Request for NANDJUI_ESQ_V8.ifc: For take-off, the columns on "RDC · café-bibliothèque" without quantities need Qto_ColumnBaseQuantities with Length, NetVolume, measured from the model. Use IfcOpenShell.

First a look at what the model holds.

```python
import ifcopenshell
import ifcopenshell.util.element
import ifcopenshell.util.unit

model = ifcopenshell.open("NANDJUI_ESQ_V8.ifc")
print(model.schema)
for unit_type in ("LENGTHUNIT", "AREAUNIT", "VOLUMEUNIT"):
    print(unit_type, ifcopenshell.util.unit.calculate_unit_scale(model, unit_type))
storey = next(s for s in model.by_type("IfcBuildingStorey") if s.Name == "RDC · café-bibliothèque")
columns = [e for e in ifcopenshell.util.element.get_decomposition(storey) if e.is_a("IfcColumn")]
for e in sorted(columns, key=lambda e: e.id()):
    print(e.id(), e.is_a(), e.Name, list(ifcopenshell.util.element.get_psets(e, qtos_only=True)), sep=" | ")
```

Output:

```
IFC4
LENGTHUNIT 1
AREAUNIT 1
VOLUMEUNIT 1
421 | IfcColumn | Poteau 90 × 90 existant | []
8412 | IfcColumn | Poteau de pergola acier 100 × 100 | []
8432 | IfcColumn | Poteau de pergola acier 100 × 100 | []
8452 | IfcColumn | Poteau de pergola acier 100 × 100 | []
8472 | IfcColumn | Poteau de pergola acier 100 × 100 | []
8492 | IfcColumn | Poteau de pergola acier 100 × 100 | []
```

```python
import ifcopenshell
import ifcopenshell.api.pset
import ifcopenshell.geom
import ifcopenshell.util.element
import ifcopenshell.util.shape
import ifcopenshell.util.unit

model = ifcopenshell.open("NANDJUI_ESQ_V8.ifc")
unit_scale = ifcopenshell.util.unit.calculate_unit_scale(model)
volume_scale = ifcopenshell.util.unit.calculate_unit_scale(model, "VOLUMEUNIT")
settings = ifcopenshell.geom.settings()

storey = next(s for s in model.by_type("IfcBuildingStorey") if s.Name == "RDC · café-bibliothèque")
columns = [e for e in ifcopenshell.util.element.get_decomposition(storey) if e.is_a("IfcColumn")]

for e in sorted(columns, key=lambda e: e.id()):
    if ifcopenshell.util.element.get_psets(e, qtos_only=True, should_inherit=False):
        continue
    # Geometry comes back in metres, in the element's own axes.
    shape = ifcopenshell.geom.create_shape(settings, e)
    values = {
        "Length": ifcopenshell.util.shape.get_z(shape.geometry) / unit_scale,
        "NetVolume": ifcopenshell.util.shape.get_volume(shape.geometry) / volume_scale,
    }
    qto = ifcopenshell.api.pset.add_qto(model, product=e, name="Qto_ColumnBaseQuantities")
    ifcopenshell.api.pset.edit_qto(model, qto=qto, properties=values)
    print(e.id(), {k: round(v, 3) for k, v in values.items()})

model.write("NANDJUI_ESQ_V8_edited.ifc")
```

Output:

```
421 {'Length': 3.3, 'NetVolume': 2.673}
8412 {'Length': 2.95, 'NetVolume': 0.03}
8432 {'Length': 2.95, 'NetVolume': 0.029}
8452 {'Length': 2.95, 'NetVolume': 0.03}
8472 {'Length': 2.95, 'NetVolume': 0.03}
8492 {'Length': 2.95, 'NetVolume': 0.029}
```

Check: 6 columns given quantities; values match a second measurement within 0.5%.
